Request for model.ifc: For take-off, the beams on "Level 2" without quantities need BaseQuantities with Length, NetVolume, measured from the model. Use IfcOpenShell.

First a look at what the model holds.

```python
import ifcopenshell
import ifcopenshell.util.element
import ifcopenshell.util.unit

model = ifcopenshell.open("model.ifc")
print(model.schema)
for unit_type in ("LENGTHUNIT", "AREAUNIT", "VOLUMEUNIT"):
    print(unit_type, ifcopenshell.util.unit.calculate_unit_scale(model, unit_type))
storey = next(s for s in model.by_type("IfcBuildingStorey") if s.Name == "Level 2")
beams = [e for e in ifcopenshell.util.element.get_decomposition(storey) if e.is_a("IfcBeam")]
for e in sorted(beams, key=lambda e: e.id()):
    print(e.id(), e.is_a(), e.Name, list(ifcopenshell.util.element.get_psets(e, qtos_only=True)), sep=" | ")
```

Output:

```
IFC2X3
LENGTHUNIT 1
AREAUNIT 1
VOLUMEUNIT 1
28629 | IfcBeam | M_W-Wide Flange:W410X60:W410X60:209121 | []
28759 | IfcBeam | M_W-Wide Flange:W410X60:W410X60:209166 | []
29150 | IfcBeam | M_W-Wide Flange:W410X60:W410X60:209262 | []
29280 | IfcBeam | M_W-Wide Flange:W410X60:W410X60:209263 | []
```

```python
import ifcopenshell
import ifcopenshell.api.pset
import ifcopenshell.geom
import ifcopenshell.util.element
import ifcopenshell.util.shape
import ifcopenshell.util.unit

model = ifcopenshell.open("model.ifc")
unit_scale = ifcopenshell.util.unit.calculate_unit_scale(model)
volume_scale = ifcopenshell.util.unit.calculate_unit_scale(model, "VOLUMEUNIT")
settings = ifcopenshell.geom.settings()

storey = next(s for s in model.by_type("IfcBuildingStorey") if s.Name == "Level 2")
beams = [e for e in ifcopenshell.util.element.get_decomposition(storey) if e.is_a("IfcBeam")]

for e in sorted(beams, key=lambda e: e.id()):
    if ifcopenshell.util.element.get_psets(e, qtos_only=True, should_inherit=False):
        continue
    # Geometry comes back in metres, in the element's own axes.
    shape = ifcopenshell.geom.create_shape(settings, e)
    values = {
        "Length": ifcopenshell.util.shape.get_max_xyz(shape.geometry) / unit_scale,
        "NetVolume": ifcopenshell.util.shape.get_volume(shape.geometry) / volume_scale,
    }
    qto = ifcopenshell.api.pset.add_qto(model, product=e, name="BaseQuantities")
    ifcopenshell.api.pset.edit_qto(model, qto=qto, properties=values)
    print(e.id(), {k: round(v, 3) for k, v in values.items()})

model.write("model_rev.ifc")
```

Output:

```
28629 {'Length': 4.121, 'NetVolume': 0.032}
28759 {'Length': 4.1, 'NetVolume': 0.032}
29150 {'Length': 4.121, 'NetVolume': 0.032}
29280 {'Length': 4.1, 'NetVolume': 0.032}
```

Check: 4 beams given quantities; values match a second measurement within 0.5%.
